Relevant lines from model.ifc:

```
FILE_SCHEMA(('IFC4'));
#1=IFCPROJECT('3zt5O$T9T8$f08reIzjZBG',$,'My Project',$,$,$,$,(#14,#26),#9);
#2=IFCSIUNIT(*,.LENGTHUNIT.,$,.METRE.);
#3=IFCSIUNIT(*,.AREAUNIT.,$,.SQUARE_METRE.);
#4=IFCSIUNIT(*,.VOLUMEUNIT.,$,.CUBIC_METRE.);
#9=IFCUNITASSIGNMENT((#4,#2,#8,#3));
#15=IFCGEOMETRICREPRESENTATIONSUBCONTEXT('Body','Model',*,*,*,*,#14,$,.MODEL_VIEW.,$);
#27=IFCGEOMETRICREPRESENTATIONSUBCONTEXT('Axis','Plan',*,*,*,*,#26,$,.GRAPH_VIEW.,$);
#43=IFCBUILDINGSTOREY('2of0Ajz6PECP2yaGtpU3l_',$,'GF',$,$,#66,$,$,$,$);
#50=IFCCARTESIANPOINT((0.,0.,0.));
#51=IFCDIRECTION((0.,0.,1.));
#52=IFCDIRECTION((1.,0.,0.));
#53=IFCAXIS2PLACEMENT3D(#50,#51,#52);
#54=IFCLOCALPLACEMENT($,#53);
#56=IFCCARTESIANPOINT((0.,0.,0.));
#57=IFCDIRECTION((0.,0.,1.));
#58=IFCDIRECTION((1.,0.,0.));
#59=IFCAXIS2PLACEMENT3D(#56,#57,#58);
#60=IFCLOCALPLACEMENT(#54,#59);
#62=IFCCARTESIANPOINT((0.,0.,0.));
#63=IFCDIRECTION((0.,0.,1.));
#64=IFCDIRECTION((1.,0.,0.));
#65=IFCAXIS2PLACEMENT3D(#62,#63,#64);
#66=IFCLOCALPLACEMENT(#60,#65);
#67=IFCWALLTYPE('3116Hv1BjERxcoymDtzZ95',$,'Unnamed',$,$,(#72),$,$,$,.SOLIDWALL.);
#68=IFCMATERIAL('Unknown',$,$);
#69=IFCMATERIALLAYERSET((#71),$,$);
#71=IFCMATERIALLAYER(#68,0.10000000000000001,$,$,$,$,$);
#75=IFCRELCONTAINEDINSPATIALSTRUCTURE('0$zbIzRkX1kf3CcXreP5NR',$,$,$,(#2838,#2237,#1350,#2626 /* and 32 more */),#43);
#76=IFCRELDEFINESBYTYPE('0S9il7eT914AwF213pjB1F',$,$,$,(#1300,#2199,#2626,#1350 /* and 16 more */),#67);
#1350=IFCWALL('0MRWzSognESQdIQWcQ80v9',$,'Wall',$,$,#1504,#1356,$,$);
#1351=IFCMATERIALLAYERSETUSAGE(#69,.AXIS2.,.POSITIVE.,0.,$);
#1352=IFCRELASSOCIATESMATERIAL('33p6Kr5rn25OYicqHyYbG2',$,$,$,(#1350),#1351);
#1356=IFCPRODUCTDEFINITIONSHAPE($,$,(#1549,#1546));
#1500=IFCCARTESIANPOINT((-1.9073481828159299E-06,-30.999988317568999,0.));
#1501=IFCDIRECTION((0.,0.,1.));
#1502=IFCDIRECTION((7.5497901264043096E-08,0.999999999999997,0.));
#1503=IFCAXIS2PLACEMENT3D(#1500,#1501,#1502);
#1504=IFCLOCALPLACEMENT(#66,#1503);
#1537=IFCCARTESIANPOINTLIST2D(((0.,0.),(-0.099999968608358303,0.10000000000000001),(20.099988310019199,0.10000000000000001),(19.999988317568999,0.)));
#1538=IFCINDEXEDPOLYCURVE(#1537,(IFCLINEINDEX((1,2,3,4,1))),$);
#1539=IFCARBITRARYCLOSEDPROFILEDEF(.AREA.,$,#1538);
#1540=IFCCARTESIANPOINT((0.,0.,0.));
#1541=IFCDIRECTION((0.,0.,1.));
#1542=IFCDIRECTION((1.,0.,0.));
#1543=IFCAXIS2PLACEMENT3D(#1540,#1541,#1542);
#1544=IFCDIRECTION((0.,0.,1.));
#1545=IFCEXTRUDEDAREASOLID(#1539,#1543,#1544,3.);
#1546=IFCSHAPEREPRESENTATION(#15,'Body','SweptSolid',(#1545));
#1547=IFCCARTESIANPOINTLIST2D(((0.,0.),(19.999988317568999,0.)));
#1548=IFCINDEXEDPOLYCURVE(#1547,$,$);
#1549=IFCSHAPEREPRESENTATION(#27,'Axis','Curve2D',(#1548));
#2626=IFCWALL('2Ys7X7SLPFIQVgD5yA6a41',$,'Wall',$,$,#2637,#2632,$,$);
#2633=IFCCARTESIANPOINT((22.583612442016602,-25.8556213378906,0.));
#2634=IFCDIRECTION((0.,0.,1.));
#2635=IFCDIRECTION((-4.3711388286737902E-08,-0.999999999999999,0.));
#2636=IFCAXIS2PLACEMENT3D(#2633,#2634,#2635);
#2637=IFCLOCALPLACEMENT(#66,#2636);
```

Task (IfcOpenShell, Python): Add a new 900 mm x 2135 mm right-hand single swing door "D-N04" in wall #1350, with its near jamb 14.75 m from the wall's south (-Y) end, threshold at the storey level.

```python
import numpy as np
import ifcopenshell
import ifcopenshell.api.feature
import ifcopenshell.api.geometry
import ifcopenshell.api.root
import ifcopenshell.api.spatial
import ifcopenshell.geom
import ifcopenshell.util.element
import ifcopenshell.util.placement
import ifcopenshell.util.representation
import ifcopenshell.util.shape
import ifcopenshell.util.unit

model = ifcopenshell.open("model.ifc")
unit_scale = ifcopenshell.util.unit.calculate_unit_scale(model)
settings = ifcopenshell.geom.settings()


def volume(element):
    """Net volume in cubic metres, openings subtracted."""
    shape = ifcopenshell.geom.create_shape(settings, element)
    return ifcopenshell.util.shape.get_volume(shape.geometry)


wall = model.by_id(1350)
storey = ifcopenshell.util.element.get_container(wall, ifc_class="IfcBuildingStorey")
context = ifcopenshell.util.representation.get_context(model, "Model", "Body", "MODEL_VIEW")
before = volume(wall)

width, height, from_end, sill = 0.9, 2.135, 14.75, 0.0  # metres

# The wall runs along its own X axis, and the end named is its -X end.
wall_shape = ifcopenshell.geom.create_shape(settings, wall)
x, y, z = ifcopenshell.util.shape.get_vertices(wall_shape.geometry).T
start = x.min() + from_end
face, thickness = float(y.min()), float(y.max() - y.min())
wall_matrix = ifcopenshell.util.placement.get_local_placement(wall.ObjectPlacement)
level = ifcopenshell.util.placement.get_local_placement(storey.ObjectPlacement)[2, 3]


def in_wall(x, y):
    """Placement at x, y metres in the wall's axes, at sill height."""
    matrix = wall_matrix.copy()
    matrix[:, 3] = wall_matrix @ np.array([x / unit_scale, y / unit_scale, 0.0, 1.0])
    matrix[2, 3] = level + sill / unit_scale
    return matrix


# Opening: a box that overshoots both wall faces by 50 mm.
opening = ifcopenshell.api.root.create_entity(model, ifc_class="IfcOpeningElement", predefined_type="OPENING")
box = ifcopenshell.api.geometry.add_wall_representation(
    model, context=context, length=width, height=height, thickness=thickness + 0.1
)
ifcopenshell.api.geometry.assign_representation(model, product=opening, representation=box)
ifcopenshell.api.geometry.edit_object_placement(model, product=opening, matrix=in_wall(start, face - 0.05), is_si=False)
ifcopenshell.api.feature.add_feature(model, feature=opening, element=wall)

door = ifcopenshell.api.root.create_entity(model, ifc_class="IfcDoor", name="D-N04", predefined_type="DOOR")
door.OverallWidth, door.OverallHeight = width / unit_scale, height / unit_scale
door.OperationType = "SINGLE_SWING_RIGHT"
body = ifcopenshell.api.geometry.add_door_representation(
    model,
    context=context,
    overall_width=door.OverallWidth,
    overall_height=door.OverallHeight,
    operation_type="SINGLE_SWING_RIGHT",
    lining_properties={"LiningDepth": thickness / unit_scale, "ThresholdDepth": thickness / unit_scale},
)
ifcopenshell.api.geometry.assign_representation(model, product=door, representation=body)
ifcopenshell.api.spatial.assign_container(model, products=[door], relating_structure=storey)
ifcopenshell.api.feature.add_filling(model, opening=opening, element=door)

# The lining spans the wall, so the door starts at the wall face.
ifcopenshell.api.geometry.edit_object_placement(model, product=door, matrix=in_wall(start, face), is_si=False)

after = volume(wall)

print(f"wall volume {before:.3f} -> {after:.3f} m3")

model.write("model_v2.ifc")
```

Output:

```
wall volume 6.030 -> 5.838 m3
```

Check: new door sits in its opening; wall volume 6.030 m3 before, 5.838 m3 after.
